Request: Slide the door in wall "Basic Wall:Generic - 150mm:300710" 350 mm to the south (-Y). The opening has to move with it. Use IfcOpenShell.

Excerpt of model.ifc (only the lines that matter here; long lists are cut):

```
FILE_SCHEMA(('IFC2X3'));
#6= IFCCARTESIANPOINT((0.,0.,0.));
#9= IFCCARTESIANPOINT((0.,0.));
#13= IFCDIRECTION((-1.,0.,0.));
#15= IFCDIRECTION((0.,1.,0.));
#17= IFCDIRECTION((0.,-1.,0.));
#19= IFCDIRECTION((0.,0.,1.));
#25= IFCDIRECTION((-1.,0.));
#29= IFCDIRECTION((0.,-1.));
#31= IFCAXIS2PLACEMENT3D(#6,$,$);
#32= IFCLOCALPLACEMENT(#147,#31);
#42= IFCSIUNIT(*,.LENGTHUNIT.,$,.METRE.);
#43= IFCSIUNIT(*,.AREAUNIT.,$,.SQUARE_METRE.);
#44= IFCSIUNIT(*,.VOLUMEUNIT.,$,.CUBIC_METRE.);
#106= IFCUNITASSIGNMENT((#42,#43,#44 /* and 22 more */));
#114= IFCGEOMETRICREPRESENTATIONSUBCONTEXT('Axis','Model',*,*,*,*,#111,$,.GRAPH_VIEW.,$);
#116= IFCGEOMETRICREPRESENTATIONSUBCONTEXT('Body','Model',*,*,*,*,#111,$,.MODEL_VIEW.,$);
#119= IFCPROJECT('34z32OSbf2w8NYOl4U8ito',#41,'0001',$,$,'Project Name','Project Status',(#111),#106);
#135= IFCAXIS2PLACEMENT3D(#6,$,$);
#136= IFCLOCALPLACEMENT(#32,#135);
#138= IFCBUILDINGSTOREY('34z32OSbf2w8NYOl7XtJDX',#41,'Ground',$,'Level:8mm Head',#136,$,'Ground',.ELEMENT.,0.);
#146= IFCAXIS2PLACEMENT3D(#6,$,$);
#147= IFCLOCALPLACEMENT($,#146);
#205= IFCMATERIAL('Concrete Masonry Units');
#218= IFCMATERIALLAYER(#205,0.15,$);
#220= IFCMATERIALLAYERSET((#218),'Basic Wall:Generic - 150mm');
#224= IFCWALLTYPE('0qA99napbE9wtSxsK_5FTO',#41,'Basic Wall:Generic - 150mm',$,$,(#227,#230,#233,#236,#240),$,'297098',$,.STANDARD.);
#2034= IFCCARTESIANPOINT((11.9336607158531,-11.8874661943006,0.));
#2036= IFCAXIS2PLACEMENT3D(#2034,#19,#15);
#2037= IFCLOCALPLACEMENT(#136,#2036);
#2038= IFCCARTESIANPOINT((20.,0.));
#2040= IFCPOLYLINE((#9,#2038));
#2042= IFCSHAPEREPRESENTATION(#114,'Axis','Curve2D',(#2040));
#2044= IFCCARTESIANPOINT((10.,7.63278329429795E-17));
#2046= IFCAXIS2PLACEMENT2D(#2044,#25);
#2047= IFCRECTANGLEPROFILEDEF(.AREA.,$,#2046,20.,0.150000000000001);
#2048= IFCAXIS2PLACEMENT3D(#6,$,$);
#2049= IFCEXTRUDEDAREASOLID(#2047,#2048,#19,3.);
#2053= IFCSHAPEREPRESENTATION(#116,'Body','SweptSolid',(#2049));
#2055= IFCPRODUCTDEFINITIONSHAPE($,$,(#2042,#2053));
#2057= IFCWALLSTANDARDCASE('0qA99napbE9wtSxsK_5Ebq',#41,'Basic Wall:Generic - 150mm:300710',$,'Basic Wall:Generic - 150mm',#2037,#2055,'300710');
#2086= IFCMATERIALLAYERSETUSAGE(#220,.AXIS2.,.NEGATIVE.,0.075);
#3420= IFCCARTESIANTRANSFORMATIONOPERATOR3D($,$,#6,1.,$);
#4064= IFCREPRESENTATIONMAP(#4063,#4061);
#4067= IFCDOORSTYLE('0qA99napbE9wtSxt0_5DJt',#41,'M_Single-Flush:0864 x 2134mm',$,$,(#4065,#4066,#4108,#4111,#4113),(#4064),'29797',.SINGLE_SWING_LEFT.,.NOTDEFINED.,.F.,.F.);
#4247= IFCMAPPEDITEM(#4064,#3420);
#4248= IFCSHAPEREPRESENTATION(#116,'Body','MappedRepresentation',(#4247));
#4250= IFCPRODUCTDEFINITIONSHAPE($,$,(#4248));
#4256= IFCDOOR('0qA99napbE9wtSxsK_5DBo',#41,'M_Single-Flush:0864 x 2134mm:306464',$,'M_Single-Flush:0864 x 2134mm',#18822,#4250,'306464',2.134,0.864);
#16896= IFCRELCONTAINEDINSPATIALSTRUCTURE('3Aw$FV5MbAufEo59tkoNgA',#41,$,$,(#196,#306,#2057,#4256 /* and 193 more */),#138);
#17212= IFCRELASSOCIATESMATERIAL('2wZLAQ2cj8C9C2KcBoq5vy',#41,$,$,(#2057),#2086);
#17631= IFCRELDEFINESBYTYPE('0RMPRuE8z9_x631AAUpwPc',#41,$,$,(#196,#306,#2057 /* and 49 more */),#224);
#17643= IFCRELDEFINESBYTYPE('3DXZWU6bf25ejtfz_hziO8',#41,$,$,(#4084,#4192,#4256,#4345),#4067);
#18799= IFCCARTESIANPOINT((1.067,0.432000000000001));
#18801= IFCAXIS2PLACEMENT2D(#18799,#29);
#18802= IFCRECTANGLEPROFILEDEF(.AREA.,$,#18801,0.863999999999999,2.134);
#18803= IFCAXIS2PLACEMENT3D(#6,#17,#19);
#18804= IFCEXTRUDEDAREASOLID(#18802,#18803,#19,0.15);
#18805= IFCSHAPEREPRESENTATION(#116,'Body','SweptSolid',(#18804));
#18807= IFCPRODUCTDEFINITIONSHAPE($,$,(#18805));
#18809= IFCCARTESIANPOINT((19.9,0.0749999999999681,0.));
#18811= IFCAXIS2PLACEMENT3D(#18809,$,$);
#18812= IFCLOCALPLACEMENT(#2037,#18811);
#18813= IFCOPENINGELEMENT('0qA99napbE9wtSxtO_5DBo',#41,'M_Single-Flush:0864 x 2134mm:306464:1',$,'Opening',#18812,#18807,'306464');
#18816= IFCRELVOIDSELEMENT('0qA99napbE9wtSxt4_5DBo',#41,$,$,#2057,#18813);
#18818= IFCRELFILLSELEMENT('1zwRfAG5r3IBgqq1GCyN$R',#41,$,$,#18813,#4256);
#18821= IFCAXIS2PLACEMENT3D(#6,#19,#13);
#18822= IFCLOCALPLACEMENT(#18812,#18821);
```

```python
import ifcopenshell
import ifcopenshell.api.geometry
import ifcopenshell.util.placement
import ifcopenshell.util.unit

model = ifcopenshell.open("model.ifc")
unit_scale = ifcopenshell.util.unit.calculate_unit_scale(model)

door = model.by_guid("0qA99napbE9wtSxsK_5DBo")
opening = door.FillsVoids[0].RelatingOpeningElement
wall = opening.VoidsElements[0].RelatingBuildingElement

wall_matrix = ifcopenshell.util.placement.get_local_placement(wall.ObjectPlacement)
shift = wall_matrix[:3, 0] * -0.35 / unit_scale
before = ifcopenshell.util.placement.get_local_placement(door.ObjectPlacement)[:3, 3].copy()

# The door is placed relative to its opening, so it follows when the opening moves.
matrix = ifcopenshell.util.placement.get_local_placement(opening.ObjectPlacement)
matrix[:3, 3] += shift
ifcopenshell.api.geometry.edit_object_placement(
    model, product=opening, matrix=matrix, is_si=False, should_transform_children=True
)

after = ifcopenshell.util.placement.get_local_placement(door.ObjectPlacement)[:3, 3]
print("door moved by", (after - before).round(3) + 0.0)

model.write("model_v2.ifc")
```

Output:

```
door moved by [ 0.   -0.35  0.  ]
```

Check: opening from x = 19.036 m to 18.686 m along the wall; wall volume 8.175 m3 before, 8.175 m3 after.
